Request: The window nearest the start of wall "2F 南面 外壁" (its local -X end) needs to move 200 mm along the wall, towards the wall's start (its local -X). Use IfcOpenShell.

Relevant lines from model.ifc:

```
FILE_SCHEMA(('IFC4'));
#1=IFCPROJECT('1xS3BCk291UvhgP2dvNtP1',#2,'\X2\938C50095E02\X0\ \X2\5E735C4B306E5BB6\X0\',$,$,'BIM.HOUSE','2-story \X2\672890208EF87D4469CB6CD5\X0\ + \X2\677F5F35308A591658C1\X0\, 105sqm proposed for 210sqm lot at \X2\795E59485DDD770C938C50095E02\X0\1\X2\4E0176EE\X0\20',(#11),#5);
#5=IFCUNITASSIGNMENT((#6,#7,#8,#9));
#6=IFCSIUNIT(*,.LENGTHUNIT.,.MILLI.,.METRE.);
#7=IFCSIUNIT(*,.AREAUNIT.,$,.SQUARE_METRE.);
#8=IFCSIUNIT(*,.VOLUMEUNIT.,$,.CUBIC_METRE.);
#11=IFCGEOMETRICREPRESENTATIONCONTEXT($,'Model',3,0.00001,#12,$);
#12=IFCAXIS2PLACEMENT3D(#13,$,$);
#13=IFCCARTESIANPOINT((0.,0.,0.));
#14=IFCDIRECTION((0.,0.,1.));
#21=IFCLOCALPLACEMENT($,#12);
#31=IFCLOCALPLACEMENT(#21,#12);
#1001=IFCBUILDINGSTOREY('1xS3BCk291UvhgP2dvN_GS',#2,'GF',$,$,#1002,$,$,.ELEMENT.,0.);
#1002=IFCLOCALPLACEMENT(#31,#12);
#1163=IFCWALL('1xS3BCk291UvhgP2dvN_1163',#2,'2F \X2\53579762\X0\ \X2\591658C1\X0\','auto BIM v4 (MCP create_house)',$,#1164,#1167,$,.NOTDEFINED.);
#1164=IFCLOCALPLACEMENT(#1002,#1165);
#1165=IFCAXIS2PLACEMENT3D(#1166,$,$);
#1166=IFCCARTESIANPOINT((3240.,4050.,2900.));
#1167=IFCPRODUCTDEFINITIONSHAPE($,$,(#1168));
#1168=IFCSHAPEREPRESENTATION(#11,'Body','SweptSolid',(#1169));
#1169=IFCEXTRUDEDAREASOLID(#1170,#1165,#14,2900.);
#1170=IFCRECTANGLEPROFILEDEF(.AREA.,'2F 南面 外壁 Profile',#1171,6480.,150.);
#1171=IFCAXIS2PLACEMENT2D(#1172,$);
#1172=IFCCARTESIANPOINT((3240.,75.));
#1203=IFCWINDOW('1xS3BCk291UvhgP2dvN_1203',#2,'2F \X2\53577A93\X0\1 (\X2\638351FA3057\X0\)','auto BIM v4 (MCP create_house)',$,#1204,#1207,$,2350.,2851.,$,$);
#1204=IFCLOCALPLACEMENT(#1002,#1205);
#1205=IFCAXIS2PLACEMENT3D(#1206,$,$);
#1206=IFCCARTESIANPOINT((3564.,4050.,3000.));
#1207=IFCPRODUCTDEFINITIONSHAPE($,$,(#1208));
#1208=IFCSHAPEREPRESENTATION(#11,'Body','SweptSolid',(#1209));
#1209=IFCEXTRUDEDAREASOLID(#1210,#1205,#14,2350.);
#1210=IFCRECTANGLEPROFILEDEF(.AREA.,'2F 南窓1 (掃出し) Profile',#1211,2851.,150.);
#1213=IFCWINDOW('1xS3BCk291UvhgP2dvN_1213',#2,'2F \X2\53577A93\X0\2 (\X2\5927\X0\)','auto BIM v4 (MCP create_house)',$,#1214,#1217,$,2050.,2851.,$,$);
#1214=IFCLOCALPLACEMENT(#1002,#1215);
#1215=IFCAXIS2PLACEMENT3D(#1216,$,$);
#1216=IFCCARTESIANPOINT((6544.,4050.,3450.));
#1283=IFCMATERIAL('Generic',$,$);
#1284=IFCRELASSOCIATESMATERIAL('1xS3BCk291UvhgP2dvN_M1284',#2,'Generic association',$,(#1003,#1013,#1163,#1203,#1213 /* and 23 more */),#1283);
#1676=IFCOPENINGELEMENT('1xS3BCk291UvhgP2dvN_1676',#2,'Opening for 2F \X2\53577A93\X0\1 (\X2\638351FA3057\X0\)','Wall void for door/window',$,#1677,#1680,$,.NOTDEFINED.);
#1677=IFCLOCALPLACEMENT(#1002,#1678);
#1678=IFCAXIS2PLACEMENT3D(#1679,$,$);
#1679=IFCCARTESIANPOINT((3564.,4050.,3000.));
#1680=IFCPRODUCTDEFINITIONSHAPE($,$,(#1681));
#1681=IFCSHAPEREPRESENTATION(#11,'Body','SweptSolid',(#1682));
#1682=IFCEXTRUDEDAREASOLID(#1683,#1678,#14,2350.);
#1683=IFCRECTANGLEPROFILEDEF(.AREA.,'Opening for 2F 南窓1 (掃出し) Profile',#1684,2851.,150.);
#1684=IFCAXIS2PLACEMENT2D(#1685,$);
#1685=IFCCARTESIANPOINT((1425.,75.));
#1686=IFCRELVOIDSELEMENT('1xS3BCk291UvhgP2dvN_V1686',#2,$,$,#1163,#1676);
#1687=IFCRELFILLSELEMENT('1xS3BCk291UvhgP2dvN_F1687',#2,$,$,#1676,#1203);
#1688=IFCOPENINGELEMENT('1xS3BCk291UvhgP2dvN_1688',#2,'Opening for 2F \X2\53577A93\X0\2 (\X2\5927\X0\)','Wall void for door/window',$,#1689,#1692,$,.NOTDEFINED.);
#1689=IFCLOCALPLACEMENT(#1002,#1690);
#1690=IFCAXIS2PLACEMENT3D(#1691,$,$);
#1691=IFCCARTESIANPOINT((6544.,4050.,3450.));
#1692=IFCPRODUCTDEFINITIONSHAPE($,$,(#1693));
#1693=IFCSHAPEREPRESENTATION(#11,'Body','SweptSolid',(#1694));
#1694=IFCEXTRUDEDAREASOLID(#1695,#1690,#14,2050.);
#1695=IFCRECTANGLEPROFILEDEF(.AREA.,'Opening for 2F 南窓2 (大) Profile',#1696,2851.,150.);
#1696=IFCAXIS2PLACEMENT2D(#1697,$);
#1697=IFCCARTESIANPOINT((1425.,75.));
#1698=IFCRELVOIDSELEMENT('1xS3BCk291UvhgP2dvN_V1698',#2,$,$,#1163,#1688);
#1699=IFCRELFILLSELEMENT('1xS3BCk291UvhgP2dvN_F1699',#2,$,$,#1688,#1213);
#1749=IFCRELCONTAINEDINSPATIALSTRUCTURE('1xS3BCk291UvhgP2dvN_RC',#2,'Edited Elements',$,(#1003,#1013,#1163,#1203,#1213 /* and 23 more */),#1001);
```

```python
import ifcopenshell
import ifcopenshell.api.geometry
import ifcopenshell.util.placement

model = ifcopenshell.open("model.ifc")

window = model.by_guid("1xS3BCk291UvhgP2dvN_1203")
opening = window.FillsVoids[0].RelatingOpeningElement
wall = opening.VoidsElements[0].RelatingBuildingElement

wall_matrix = ifcopenshell.util.placement.get_local_placement(wall.ObjectPlacement)
shift = wall_matrix[:3, 0] * -200.0
before = ifcopenshell.util.placement.get_local_placement(window.ObjectPlacement)[:3, 3].copy()

# The window is not placed relative to its opening, so move both.
for product in (opening, window):
    matrix = ifcopenshell.util.placement.get_local_placement(product.ObjectPlacement)
    matrix[:3, 3] += shift
    ifcopenshell.api.geometry.edit_object_placement(model, product=product, matrix=matrix, is_si=False)

after = ifcopenshell.util.placement.get_local_placement(window.ObjectPlacement)[:3, 3]
print("window moved by", (after - before).round(3) + 0.0)

model.write("model_rev.ifc")
```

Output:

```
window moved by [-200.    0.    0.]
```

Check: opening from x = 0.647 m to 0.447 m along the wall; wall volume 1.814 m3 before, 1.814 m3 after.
